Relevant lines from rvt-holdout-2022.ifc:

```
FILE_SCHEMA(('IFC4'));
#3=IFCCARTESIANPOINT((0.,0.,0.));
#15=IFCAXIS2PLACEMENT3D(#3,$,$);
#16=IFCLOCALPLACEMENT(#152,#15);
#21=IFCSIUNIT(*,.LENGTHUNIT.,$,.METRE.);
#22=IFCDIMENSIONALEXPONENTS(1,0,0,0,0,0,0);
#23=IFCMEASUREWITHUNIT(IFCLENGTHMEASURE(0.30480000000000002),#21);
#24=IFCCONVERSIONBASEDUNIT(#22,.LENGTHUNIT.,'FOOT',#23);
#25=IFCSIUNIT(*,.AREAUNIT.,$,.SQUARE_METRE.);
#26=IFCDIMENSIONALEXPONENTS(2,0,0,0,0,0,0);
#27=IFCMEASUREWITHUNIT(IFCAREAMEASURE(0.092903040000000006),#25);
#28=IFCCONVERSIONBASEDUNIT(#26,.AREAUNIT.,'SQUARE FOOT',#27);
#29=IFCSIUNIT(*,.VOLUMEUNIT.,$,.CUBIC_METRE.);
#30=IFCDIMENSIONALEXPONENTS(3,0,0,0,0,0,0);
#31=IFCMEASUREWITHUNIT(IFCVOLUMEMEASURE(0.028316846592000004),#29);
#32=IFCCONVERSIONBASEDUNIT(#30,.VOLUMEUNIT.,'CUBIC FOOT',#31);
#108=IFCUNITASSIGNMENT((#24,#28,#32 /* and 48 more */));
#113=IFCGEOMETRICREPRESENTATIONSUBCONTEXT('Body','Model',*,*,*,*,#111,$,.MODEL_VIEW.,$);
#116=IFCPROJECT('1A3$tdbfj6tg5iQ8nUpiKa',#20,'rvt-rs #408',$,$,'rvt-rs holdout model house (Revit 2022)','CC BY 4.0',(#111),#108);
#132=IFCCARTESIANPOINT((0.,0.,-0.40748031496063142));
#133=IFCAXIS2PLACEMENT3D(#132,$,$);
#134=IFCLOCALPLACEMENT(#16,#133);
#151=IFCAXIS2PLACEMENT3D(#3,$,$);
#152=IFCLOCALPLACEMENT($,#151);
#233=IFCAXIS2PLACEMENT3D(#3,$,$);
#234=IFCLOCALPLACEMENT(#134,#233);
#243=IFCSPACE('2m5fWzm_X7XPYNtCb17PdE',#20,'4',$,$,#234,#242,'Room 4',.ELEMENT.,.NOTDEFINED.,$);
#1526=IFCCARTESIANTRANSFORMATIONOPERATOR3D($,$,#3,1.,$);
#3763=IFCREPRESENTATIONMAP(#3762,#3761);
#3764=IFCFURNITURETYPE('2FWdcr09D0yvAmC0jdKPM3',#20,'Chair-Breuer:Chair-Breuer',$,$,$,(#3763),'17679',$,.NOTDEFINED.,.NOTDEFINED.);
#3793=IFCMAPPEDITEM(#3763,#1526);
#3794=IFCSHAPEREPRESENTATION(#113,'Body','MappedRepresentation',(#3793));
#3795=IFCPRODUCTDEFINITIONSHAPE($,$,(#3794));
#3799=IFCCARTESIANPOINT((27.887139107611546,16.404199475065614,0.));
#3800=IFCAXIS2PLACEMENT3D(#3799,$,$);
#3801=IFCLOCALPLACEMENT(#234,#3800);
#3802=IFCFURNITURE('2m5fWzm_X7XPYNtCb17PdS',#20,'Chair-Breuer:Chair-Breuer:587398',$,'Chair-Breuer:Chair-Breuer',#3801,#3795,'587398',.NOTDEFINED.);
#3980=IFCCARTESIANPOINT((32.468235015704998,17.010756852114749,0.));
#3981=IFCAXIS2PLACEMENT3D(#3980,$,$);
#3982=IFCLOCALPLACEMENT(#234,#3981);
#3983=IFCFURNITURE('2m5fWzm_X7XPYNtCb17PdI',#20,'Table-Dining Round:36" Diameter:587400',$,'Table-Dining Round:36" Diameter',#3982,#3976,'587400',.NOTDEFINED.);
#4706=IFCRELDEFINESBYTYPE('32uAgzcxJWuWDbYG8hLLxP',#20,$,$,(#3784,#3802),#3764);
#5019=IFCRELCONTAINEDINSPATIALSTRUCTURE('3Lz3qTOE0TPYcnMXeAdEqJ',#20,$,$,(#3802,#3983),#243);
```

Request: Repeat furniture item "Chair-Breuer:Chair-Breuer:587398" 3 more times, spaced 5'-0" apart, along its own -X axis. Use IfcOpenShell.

```python
import ifcopenshell
import ifcopenshell.api.geometry
import ifcopenshell.api.root
import ifcopenshell.util.element
import ifcopenshell.util.placement
import ifcopenshell.util.unit

model = ifcopenshell.open("rvt-holdout-2022.ifc")
unit_scale = ifcopenshell.util.unit.calculate_unit_scale(model)


def reuse_history(source, copy):
    """copy_class also copies each property set's owner history, people and application; keep the originals."""
    for rel in copy.IsDefinedBy:
        if rel.is_a("IfcRelDefinesByProperties") and (history := rel.RelatingPropertyDefinition.OwnerHistory):
            rel.RelatingPropertyDefinition.OwnerHistory = source.OwnerHistory
            ifcopenshell.util.element.remove_deep2(model, history)


source = model.by_guid("2m5fWzm_X7XPYNtCb17PdS")
base = ifcopenshell.util.placement.get_local_placement(source.ObjectPlacement)
step = -base[:3, 0] * 60 * 0.0254 / unit_scale

for i in range(1, 4):
    copy = ifcopenshell.api.root.copy_class(model, product=source)
    copy.Representation = ifcopenshell.util.element.copy_deep(
        model, source.Representation, exclude=["IfcGeometricRepresentationContext", "IfcRepresentationMap"]
    )
    copy.Name = "Chair-Breuer:Chair-Breuer"
    copy.Tag = None
    reuse_history(source, copy)
    matrix = base.copy()
    matrix[:3, 3] += i * step
    print("added at", matrix[:3, 3].round(3) + 0.0)
    ifcopenshell.api.geometry.edit_object_placement(model, product=copy, matrix=matrix, is_si=False)

model.write("rvt-holdout-2022_v2.ifc")
```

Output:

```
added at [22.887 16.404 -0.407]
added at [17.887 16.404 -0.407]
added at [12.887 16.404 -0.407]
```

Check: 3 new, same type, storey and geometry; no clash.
